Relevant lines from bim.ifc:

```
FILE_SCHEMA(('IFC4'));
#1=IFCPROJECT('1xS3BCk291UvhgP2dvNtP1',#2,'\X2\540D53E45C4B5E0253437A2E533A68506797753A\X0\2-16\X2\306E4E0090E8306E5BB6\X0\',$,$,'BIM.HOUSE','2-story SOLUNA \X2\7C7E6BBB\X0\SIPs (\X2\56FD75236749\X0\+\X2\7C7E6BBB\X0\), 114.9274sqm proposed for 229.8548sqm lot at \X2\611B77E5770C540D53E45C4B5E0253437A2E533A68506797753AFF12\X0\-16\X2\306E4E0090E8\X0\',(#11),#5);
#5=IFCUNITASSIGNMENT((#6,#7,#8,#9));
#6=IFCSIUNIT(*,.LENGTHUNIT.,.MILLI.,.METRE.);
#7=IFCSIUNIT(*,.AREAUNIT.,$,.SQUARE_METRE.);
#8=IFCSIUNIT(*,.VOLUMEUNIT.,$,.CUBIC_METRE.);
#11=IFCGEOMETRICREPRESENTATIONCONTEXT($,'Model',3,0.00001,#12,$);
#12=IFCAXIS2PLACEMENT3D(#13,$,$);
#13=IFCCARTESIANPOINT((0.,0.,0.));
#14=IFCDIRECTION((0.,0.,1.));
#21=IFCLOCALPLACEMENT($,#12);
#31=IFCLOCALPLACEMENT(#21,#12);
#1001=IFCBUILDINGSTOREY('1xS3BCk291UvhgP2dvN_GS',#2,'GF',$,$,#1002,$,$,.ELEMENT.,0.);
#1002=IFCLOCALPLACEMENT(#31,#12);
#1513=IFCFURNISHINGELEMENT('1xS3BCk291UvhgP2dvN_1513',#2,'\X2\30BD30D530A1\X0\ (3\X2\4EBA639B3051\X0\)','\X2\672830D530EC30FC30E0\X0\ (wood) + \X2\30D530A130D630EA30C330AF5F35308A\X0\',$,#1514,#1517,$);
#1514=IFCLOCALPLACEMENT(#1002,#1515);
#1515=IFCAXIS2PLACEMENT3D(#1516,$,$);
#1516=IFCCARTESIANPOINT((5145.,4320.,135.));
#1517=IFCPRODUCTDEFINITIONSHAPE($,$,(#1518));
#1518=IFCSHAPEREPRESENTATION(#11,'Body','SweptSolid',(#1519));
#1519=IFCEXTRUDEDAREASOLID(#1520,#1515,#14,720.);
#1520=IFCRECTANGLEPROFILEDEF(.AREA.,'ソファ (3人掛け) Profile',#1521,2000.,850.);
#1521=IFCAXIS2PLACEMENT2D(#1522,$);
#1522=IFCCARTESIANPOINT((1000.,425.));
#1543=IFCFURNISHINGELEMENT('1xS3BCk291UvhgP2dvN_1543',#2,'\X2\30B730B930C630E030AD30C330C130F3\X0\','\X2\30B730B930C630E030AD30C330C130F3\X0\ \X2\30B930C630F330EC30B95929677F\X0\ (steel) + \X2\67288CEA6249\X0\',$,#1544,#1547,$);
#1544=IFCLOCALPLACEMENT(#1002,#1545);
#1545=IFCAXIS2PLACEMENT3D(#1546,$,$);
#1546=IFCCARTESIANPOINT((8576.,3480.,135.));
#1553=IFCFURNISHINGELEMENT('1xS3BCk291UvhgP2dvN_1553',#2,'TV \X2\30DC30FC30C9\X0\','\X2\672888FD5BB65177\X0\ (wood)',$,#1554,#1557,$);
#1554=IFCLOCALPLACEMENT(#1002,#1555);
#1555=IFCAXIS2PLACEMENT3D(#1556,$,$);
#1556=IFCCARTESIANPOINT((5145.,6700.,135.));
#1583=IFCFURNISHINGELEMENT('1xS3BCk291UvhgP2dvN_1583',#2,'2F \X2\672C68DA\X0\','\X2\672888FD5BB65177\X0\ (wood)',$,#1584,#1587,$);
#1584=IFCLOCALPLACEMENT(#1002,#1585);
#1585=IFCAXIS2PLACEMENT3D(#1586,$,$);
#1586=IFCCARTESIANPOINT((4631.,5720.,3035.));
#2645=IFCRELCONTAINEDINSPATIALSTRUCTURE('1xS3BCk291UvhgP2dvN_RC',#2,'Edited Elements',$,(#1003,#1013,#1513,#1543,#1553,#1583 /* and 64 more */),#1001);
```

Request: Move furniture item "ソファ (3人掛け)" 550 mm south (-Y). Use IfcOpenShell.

```python
import ifcopenshell
import ifcopenshell.api.geometry
import ifcopenshell.util.placement

model = ifcopenshell.open("bim.ifc")

item = model.by_guid("1xS3BCk291UvhgP2dvN_1513")
matrix = ifcopenshell.util.placement.get_local_placement(item.ObjectPlacement)
matrix[1, 3] -= 550.0
ifcopenshell.api.geometry.edit_object_placement(model, product=item, matrix=matrix, is_si=False)

print(ifcopenshell.util.placement.get_local_placement(item.ObjectPlacement).round(3) + 0.0)

model.write("bim_edited.ifc")
```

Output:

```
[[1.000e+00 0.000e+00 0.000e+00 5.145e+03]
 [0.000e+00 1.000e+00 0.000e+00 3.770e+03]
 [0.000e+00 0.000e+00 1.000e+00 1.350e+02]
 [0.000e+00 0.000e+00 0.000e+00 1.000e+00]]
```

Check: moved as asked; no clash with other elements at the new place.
